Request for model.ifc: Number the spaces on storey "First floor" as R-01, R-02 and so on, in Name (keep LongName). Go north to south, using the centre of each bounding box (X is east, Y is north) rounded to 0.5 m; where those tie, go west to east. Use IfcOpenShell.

First a look at what the model holds.

```python
import ifcopenshell
import ifcopenshell.util.element
import ifcopenshell.util.placement

model = ifcopenshell.open("model.ifc")
print(model.schema)
storey = next(s for s in model.by_type("IfcBuildingStorey") if s.Name == "First floor")
spaces = [e for e in ifcopenshell.util.element.get_decomposition(storey) if e.is_a("IfcSpace")]
for e in sorted(spaces, key=lambda e: e.id()):
    origin = ifcopenshell.util.placement.get_local_placement(e.ObjectPlacement)[:3, 3]
    print(e.id(), e.Name, e.LongName, origin.round(2) + 0.0, sep=" | ")
```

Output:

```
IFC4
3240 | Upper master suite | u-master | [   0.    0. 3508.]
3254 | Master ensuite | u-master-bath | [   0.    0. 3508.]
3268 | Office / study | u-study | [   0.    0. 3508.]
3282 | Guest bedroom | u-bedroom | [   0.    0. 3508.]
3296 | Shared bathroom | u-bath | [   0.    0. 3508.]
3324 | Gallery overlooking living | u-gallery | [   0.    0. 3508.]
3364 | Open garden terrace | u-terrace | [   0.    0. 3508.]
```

```python
import ifcopenshell
import ifcopenshell.geom
import ifcopenshell.util.element
import ifcopenshell.util.shape

model = ifcopenshell.open("model.ifc")
settings = ifcopenshell.geom.settings()
settings.set("use-world-coords", True)


def centre(element):
    shape = ifcopenshell.geom.create_shape(settings, element)
    return ifcopenshell.util.shape.get_bbox_centroid(shape.geometry)


storey = next(s for s in model.by_type("IfcBuildingStorey") if s.Name == "First floor")
spaces = [e for e in ifcopenshell.util.element.get_decomposition(storey) if e.is_a("IfcSpace")]

# Insertion points can sit at a corner or the storey origin, so sort by the geometry (in metres).
centres = {e: centre(e) for e in spaces}
spaces.sort(key=lambda e: (-round(centres[e][1] / 0.5), centres[e][0]))

for i, e in enumerate(spaces, start=1):
    number = f"R-{i:02d}"
    e.Name = number
    print(e.id(), number)

model.write("model_updated.ifc")
```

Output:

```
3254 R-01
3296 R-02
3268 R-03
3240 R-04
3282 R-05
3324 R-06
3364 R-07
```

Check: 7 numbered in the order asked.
